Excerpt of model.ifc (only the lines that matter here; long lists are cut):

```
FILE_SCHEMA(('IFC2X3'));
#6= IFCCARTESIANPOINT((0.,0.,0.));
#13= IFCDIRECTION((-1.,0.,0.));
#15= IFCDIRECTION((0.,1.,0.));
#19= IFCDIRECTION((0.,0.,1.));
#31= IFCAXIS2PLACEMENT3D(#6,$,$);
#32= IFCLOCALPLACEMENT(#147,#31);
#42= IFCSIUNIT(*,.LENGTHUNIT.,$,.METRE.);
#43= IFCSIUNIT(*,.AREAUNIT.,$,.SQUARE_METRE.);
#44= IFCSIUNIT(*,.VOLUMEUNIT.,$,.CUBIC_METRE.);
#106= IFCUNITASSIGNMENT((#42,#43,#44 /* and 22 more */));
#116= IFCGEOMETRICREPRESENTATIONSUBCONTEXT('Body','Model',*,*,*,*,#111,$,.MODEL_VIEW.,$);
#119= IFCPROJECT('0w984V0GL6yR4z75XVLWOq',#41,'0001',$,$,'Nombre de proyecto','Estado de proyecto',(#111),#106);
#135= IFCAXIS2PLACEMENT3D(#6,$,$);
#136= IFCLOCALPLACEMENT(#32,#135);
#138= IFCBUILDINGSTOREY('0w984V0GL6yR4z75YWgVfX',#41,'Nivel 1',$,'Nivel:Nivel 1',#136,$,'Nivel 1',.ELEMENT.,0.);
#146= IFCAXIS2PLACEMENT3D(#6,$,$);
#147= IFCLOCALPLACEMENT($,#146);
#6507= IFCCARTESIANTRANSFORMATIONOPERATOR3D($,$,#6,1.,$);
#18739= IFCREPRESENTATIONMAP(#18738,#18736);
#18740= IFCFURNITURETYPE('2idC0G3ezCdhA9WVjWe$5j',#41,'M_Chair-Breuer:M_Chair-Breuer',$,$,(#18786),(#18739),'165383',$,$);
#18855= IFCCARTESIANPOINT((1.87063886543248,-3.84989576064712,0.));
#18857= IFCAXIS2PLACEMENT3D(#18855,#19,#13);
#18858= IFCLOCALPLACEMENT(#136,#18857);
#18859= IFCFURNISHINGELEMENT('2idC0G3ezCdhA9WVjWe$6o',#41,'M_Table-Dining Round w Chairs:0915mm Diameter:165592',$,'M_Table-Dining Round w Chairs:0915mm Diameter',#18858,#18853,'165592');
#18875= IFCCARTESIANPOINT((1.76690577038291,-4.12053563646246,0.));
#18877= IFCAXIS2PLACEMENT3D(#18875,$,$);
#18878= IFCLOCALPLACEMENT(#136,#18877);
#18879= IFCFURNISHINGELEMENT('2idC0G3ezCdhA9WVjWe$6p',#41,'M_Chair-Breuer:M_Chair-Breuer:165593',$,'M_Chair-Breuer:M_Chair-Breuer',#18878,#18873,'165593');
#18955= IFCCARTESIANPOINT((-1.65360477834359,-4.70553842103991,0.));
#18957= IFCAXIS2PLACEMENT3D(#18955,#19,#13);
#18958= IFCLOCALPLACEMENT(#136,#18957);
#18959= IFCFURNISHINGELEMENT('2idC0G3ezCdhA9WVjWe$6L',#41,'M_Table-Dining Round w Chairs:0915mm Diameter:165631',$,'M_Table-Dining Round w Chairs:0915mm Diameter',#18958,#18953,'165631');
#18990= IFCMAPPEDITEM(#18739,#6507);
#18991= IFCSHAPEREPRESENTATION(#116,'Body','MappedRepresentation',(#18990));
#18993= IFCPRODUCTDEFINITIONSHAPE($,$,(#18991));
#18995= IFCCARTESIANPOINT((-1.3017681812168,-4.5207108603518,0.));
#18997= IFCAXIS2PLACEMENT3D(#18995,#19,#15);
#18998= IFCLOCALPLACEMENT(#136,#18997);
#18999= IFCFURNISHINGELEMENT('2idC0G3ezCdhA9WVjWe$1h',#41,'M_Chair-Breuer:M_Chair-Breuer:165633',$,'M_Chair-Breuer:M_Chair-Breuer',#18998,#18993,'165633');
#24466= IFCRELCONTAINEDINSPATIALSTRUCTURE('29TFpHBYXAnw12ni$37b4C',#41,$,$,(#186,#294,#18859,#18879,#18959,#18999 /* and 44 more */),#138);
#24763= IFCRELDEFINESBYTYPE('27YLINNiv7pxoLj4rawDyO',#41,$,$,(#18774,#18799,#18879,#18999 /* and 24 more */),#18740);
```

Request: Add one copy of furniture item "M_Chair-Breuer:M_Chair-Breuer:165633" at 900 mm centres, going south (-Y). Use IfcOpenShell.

```python
import numpy as np
import ifcopenshell
import ifcopenshell.api.geometry
import ifcopenshell.api.root
import ifcopenshell.util.element
import ifcopenshell.util.placement
import ifcopenshell.util.unit

model = ifcopenshell.open("model.ifc")
unit_scale = ifcopenshell.util.unit.calculate_unit_scale(model)


def reuse_history(source, copy):
    """copy_class also copies each property set's owner history, people and application; keep the originals."""
    for rel in copy.IsDefinedBy:
        if rel.is_a("IfcRelDefinesByProperties") and (history := rel.RelatingPropertyDefinition.OwnerHistory):
            rel.RelatingPropertyDefinition.OwnerHistory = source.OwnerHistory
            ifcopenshell.util.element.remove_deep2(model, history)


source = model.by_guid("2idC0G3ezCdhA9WVjWe$1h")
base = ifcopenshell.util.placement.get_local_placement(source.ObjectPlacement)
step = np.array([0.0, -1.0, 0.0]) * 0.9 / unit_scale

for i in range(1, 2):
    copy = ifcopenshell.api.root.copy_class(model, product=source)
    copy.Representation = ifcopenshell.util.element.copy_deep(
        model, source.Representation, exclude=["IfcGeometricRepresentationContext", "IfcRepresentationMap"]
    )
    copy.Name = "M_Chair-Breuer:M_Chair-Breuer"
    copy.Tag = None
    reuse_history(source, copy)
    matrix = base.copy()
    matrix[:3, 3] += i * step
    print("added at", matrix[:3, 3].round(3) + 0.0)
    ifcopenshell.api.geometry.edit_object_placement(model, product=copy, matrix=matrix, is_si=False)

model.write("model_updated.ifc")
```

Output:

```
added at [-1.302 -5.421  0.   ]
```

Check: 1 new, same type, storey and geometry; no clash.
